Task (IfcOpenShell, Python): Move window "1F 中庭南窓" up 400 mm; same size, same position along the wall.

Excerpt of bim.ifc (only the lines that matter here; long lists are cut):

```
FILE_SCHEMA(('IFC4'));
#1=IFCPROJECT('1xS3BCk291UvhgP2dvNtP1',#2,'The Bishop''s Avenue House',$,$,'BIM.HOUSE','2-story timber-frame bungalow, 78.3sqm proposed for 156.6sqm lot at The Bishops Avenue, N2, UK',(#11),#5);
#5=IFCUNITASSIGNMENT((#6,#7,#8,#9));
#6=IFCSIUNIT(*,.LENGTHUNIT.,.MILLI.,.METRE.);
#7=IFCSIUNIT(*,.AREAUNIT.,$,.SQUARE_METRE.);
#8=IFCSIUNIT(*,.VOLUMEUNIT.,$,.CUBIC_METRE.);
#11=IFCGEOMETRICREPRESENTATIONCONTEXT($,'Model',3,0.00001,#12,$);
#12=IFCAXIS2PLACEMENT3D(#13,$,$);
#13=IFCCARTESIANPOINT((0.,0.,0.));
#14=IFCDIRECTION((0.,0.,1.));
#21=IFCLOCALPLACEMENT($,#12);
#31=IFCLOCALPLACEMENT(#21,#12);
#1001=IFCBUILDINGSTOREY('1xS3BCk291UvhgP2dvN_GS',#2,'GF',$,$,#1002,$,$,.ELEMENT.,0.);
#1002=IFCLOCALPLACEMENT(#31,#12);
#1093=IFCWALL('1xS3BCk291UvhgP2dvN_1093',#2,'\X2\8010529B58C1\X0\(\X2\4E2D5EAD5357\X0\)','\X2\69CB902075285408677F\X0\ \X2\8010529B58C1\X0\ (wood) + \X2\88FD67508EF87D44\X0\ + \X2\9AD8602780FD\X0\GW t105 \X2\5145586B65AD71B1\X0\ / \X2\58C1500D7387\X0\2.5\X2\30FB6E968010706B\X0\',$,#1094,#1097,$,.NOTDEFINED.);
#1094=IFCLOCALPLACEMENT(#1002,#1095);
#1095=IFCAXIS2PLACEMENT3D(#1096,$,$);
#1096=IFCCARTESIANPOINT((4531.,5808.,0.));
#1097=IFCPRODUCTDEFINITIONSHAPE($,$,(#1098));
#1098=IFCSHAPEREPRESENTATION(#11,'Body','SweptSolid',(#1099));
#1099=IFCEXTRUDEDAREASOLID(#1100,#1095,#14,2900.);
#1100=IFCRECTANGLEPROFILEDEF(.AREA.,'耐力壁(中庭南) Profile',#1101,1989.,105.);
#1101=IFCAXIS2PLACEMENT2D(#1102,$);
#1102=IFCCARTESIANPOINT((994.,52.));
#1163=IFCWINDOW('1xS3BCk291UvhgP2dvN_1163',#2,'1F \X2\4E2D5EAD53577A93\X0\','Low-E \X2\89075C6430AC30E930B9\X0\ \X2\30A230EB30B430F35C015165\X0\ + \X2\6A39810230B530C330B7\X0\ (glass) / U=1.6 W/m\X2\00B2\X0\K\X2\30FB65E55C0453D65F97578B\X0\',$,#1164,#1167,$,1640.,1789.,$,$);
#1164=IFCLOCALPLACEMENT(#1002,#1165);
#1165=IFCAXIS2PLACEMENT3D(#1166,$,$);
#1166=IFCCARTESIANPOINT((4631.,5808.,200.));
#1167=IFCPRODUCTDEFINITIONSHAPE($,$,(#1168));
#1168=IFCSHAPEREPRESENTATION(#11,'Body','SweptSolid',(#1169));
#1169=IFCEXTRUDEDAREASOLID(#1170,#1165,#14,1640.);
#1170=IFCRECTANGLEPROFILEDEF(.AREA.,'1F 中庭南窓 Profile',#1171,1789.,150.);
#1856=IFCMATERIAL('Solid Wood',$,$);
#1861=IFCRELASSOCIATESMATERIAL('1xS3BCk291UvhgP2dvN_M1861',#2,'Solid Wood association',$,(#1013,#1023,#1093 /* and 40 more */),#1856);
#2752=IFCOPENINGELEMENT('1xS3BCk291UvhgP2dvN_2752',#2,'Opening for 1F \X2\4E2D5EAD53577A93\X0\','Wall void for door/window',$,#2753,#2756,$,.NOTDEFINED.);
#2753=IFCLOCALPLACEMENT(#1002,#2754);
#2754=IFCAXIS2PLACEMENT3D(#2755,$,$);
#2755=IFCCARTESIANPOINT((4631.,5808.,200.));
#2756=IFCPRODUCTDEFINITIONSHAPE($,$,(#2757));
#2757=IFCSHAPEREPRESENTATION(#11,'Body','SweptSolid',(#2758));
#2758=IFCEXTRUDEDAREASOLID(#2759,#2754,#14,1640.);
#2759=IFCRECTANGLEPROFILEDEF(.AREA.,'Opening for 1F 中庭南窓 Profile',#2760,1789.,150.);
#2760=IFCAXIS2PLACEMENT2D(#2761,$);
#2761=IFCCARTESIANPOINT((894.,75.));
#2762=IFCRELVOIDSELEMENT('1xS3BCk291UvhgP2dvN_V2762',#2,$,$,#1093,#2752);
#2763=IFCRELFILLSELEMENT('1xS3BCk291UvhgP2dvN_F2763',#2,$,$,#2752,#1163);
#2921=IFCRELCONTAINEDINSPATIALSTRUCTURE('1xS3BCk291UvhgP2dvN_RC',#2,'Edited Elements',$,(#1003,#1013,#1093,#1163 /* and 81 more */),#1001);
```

```python
import numpy as np
import ifcopenshell
import ifcopenshell.api.geometry
import ifcopenshell.util.placement
import ifcopenshell.util.unit

model = ifcopenshell.open("bim.ifc")
unit_scale = ifcopenshell.util.unit.calculate_unit_scale(model)

window = model.by_guid("1xS3BCk291UvhgP2dvN_1163")
opening = window.FillsVoids[0].RelatingOpeningElement
dz = 400.0

shift = np.array([0.0, 0.0, dz])
# The window is not placed relative to its opening, so move both.
for product in (opening, window):
    matrix = ifcopenshell.util.placement.get_local_placement(product.ObjectPlacement)
    matrix[:3, 3] += shift
    ifcopenshell.api.geometry.edit_object_placement(model, product=product, matrix=matrix, is_si=False)

print(f"moved by {dz * unit_scale:+.3f} m")

model.write("bim_updated.ifc")
```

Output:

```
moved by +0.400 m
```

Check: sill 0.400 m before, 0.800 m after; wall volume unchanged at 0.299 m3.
